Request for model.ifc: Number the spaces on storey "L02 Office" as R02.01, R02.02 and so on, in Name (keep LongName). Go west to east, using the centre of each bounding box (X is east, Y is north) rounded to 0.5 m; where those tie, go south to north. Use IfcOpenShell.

First a look at what the model holds.

```python
import ifcopenshell
import ifcopenshell.util.element
import ifcopenshell.util.placement

model = ifcopenshell.open("model.ifc")
print(model.schema)
storey = next(s for s in model.by_type("IfcBuildingStorey") if s.Name == "L02 Office")
spaces = [e for e in ifcopenshell.util.element.get_decomposition(storey) if e.is_a("IfcSpace")]
for e in sorted(spaces, key=lambda e: e.id()):
    origin = ifcopenshell.util.placement.get_local_placement(e.ObjectPlacement)[:3, 3]
    print(e.id(), e.Name, e.LongName, origin.round(2) + 0.0, sep=" | ")
```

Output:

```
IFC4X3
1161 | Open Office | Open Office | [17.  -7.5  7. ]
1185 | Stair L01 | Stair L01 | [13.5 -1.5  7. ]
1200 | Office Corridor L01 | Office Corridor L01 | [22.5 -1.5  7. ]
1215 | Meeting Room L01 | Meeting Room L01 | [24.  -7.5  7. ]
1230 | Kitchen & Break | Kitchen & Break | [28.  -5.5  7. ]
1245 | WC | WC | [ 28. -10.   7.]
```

```python
import ifcopenshell
import ifcopenshell.geom
import ifcopenshell.util.element
import ifcopenshell.util.shape

model = ifcopenshell.open("model.ifc")
settings = ifcopenshell.geom.settings()
settings.set("use-world-coords", True)


def centre(element):
    shape = ifcopenshell.geom.create_shape(settings, element)
    return ifcopenshell.util.shape.get_bbox_centroid(shape.geometry)


storey = next(s for s in model.by_type("IfcBuildingStorey") if s.Name == "L02 Office")
spaces = [e for e in ifcopenshell.util.element.get_decomposition(storey) if e.is_a("IfcSpace")]

# Insertion points can sit at a corner or the storey origin, so sort by the geometry (in metres).
centres = {e: centre(e) for e in spaces}
spaces.sort(key=lambda e: (round(centres[e][0] / 0.5), centres[e][1]))

for i, e in enumerate(spaces, start=1):
    number = f"R02.{i:02d}"
    e.Name = number
    print(e.id(), number)

model.write("model_rev.ifc")
```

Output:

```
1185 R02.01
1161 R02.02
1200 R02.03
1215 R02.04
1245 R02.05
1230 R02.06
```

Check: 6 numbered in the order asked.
